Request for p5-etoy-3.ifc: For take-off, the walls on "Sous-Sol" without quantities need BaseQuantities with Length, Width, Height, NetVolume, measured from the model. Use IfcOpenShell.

First a look at what the model holds.

```python
import ifcopenshell
import ifcopenshell.util.element
import ifcopenshell.util.unit

model = ifcopenshell.open("p5-etoy-3.ifc")
print(model.schema)
for unit_type in ("LENGTHUNIT", "AREAUNIT", "VOLUMEUNIT"):
    print(unit_type, ifcopenshell.util.unit.calculate_unit_scale(model, unit_type))
storey = next(s for s in model.by_type("IfcBuildingStorey") if s.Name == "Sous-Sol")
walls = [e for e in ifcopenshell.util.element.get_decomposition(storey) if e.is_a("IfcWall")]
for e in sorted(walls, key=lambda e: e.id()):
    print(e.id(), e.is_a(), e.Name, list(ifcopenshell.util.element.get_psets(e, qtos_only=True)), sep=" | ")
```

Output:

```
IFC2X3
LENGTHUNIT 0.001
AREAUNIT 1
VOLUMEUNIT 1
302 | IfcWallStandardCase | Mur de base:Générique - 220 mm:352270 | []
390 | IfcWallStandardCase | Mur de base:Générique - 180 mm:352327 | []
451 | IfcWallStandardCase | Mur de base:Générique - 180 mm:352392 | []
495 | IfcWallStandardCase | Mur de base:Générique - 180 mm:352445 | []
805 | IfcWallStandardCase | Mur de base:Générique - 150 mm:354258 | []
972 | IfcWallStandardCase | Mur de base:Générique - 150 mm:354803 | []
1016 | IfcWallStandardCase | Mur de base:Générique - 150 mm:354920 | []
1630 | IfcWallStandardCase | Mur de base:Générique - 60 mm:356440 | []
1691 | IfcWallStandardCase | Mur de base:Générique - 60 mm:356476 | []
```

```python
import ifcopenshell
import ifcopenshell.api.pset
import ifcopenshell.geom
import ifcopenshell.util.element
import ifcopenshell.util.shape
import ifcopenshell.util.unit

model = ifcopenshell.open("p5-etoy-3.ifc")
unit_scale = ifcopenshell.util.unit.calculate_unit_scale(model)
volume_scale = ifcopenshell.util.unit.calculate_unit_scale(model, "VOLUMEUNIT")
settings = ifcopenshell.geom.settings()

storey = next(s for s in model.by_type("IfcBuildingStorey") if s.Name == "Sous-Sol")
walls = [e for e in ifcopenshell.util.element.get_decomposition(storey) if e.is_a("IfcWall")]

for e in sorted(walls, key=lambda e: e.id()):
    if ifcopenshell.util.element.get_psets(e, qtos_only=True, should_inherit=False):
        continue
    # Geometry comes back in metres, in the element's own axes.
    shape = ifcopenshell.geom.create_shape(settings, e)
    values = {
        "Length": ifcopenshell.util.shape.get_x(shape.geometry) / unit_scale,
        "Width": ifcopenshell.util.shape.get_y(shape.geometry) / unit_scale,
        "Height": ifcopenshell.util.shape.get_z(shape.geometry) / unit_scale,
        "NetVolume": ifcopenshell.util.shape.get_volume(shape.geometry) / volume_scale,
    }
    qto = ifcopenshell.api.pset.add_qto(model, product=e, name="BaseQuantities")
    ifcopenshell.api.pset.edit_qto(model, qto=qto, properties=values)
    print(e.id(), {k: round(v, 3) for k, v in values.items()})

model.write("p5-etoy-3-out.ifc")
```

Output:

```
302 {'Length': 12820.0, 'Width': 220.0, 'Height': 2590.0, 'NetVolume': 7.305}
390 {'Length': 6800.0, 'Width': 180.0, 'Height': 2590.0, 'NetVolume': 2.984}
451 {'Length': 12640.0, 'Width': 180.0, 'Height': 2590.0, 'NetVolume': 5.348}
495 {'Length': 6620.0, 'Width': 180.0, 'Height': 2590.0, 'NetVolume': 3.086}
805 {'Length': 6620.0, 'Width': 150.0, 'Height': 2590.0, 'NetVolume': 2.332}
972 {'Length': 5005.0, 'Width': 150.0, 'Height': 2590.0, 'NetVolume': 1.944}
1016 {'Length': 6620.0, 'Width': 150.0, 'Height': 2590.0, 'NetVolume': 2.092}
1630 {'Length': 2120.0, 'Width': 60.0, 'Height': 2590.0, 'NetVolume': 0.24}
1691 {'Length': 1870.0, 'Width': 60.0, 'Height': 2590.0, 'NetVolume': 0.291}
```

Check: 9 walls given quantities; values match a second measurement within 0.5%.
